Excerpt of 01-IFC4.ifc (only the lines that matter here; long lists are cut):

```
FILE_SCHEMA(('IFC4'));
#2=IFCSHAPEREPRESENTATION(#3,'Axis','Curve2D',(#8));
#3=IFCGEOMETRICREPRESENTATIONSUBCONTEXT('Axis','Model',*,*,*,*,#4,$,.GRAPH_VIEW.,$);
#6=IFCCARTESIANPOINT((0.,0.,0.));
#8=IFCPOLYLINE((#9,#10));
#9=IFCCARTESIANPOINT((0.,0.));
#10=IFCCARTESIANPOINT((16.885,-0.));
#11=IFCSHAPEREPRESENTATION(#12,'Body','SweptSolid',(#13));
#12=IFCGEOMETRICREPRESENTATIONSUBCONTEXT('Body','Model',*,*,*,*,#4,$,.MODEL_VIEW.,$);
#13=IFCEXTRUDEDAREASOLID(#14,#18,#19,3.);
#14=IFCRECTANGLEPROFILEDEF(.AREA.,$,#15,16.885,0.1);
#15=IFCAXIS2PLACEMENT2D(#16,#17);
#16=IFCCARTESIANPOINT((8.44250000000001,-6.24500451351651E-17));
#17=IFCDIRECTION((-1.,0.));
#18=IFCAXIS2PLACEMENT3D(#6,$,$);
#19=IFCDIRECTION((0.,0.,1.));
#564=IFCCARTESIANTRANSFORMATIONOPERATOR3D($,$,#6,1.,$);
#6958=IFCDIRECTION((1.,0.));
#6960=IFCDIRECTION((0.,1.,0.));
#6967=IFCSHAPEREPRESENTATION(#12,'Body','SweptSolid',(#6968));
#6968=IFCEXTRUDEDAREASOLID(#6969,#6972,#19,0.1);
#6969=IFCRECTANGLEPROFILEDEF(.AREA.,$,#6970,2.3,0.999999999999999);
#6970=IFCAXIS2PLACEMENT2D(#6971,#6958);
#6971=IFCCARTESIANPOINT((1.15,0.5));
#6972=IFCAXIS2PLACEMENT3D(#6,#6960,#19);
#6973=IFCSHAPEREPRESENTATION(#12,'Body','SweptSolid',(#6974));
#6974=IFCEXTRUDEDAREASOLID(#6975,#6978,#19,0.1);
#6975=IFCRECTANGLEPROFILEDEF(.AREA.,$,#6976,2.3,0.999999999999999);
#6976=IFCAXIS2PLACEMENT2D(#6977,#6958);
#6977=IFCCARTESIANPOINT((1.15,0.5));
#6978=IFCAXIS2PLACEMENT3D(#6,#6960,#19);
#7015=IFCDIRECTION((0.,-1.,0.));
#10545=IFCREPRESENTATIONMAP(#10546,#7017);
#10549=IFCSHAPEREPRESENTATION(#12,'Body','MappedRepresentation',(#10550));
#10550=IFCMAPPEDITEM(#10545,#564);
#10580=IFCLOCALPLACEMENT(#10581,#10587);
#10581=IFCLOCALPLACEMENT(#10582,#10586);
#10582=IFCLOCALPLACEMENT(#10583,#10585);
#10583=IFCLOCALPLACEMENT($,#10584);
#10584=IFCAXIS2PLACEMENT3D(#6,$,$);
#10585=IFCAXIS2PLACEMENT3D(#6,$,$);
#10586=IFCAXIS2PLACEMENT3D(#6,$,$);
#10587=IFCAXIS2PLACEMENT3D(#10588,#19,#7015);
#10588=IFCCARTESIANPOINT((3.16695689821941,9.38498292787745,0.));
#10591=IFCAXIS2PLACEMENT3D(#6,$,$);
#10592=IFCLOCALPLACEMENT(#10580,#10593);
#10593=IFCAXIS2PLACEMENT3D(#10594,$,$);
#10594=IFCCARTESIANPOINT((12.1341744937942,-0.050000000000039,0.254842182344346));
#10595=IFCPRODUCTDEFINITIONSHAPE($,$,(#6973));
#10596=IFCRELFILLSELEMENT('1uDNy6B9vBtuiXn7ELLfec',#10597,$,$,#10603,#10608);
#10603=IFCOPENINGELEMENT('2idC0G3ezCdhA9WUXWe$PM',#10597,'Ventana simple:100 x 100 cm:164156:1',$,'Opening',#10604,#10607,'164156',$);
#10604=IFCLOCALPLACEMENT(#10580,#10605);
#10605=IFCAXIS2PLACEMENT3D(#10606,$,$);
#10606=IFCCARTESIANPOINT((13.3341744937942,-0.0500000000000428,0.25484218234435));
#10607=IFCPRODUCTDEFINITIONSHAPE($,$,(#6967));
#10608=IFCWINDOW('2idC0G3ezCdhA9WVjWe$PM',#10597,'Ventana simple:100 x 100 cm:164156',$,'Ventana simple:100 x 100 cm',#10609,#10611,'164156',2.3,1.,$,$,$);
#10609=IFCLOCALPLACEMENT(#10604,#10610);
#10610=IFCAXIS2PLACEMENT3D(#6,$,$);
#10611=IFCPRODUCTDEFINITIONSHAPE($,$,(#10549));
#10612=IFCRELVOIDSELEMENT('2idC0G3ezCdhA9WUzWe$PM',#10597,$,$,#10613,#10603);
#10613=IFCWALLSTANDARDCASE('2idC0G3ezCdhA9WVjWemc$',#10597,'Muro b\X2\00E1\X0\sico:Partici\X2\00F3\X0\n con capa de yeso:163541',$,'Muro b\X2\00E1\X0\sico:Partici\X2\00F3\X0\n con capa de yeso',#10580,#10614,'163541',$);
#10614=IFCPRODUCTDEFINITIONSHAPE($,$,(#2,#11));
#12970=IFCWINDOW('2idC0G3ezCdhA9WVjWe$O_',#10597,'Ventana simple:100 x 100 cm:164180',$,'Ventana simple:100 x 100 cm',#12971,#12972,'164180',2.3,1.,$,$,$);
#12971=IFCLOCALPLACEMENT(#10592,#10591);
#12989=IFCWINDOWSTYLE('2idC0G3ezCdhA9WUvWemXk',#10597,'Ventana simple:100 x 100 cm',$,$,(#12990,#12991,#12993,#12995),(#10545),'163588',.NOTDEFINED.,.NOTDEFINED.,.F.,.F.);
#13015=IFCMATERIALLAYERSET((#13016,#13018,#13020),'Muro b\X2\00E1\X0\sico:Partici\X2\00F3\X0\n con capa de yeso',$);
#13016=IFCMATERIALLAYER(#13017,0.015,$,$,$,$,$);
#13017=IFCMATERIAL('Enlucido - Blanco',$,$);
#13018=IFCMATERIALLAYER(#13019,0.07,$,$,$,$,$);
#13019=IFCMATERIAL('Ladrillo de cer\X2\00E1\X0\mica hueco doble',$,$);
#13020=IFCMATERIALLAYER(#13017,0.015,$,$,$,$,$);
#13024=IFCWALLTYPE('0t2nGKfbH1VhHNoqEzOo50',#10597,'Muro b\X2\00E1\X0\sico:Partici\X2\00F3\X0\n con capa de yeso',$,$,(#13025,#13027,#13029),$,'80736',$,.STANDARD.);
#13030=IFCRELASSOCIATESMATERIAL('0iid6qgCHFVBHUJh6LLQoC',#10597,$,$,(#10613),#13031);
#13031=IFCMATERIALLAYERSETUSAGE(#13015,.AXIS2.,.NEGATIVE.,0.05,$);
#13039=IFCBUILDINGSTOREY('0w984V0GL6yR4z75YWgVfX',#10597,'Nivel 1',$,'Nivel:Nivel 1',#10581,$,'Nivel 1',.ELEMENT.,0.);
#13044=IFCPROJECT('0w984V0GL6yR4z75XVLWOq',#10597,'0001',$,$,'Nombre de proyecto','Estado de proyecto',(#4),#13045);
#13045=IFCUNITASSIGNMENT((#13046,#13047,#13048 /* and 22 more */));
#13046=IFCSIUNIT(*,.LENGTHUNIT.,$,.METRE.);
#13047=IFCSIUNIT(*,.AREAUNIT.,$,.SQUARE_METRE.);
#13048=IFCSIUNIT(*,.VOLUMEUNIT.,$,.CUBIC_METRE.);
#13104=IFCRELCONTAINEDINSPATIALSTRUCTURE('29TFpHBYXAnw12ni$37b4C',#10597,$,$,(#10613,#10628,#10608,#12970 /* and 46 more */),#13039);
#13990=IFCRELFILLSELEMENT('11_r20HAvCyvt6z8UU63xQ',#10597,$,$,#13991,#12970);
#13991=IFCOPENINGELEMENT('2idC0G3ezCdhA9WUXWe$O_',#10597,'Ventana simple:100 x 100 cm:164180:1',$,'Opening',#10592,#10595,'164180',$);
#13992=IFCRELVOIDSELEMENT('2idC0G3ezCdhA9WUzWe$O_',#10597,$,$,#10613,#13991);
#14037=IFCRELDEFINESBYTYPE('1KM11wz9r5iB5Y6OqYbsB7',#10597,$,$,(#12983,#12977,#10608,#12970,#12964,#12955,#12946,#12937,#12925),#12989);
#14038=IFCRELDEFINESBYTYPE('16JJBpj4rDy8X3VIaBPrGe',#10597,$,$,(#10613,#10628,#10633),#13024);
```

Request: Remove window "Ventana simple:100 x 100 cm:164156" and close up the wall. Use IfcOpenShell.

```python
import ifcopenshell
import ifcopenshell.api.feature
import ifcopenshell.api.root
import ifcopenshell.geom
import ifcopenshell.util.shape

model = ifcopenshell.open("01-IFC4.ifc")
settings = ifcopenshell.geom.settings()


def volume(element):
    """Net volume in cubic metres, openings subtracted."""
    shape = ifcopenshell.geom.create_shape(settings, element)
    return ifcopenshell.util.shape.get_volume(shape.geometry)


window = model.by_guid("2idC0G3ezCdhA9WVjWe$PM")
opening = window.FillsVoids[0].RelatingOpeningElement
wall = opening.VoidsElements[0].RelatingBuildingElement
before = volume(wall)

ifcopenshell.api.root.remove_product(model, product=window)
ifcopenshell.api.feature.remove_feature(model, feature=opening)

after = volume(wall)

print(f"wall volume {before:.3f} -> {after:.3f} m3")

model.write("01-IFC4_v2.ifc")
```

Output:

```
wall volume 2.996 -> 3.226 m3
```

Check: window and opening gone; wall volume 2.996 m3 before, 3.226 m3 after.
